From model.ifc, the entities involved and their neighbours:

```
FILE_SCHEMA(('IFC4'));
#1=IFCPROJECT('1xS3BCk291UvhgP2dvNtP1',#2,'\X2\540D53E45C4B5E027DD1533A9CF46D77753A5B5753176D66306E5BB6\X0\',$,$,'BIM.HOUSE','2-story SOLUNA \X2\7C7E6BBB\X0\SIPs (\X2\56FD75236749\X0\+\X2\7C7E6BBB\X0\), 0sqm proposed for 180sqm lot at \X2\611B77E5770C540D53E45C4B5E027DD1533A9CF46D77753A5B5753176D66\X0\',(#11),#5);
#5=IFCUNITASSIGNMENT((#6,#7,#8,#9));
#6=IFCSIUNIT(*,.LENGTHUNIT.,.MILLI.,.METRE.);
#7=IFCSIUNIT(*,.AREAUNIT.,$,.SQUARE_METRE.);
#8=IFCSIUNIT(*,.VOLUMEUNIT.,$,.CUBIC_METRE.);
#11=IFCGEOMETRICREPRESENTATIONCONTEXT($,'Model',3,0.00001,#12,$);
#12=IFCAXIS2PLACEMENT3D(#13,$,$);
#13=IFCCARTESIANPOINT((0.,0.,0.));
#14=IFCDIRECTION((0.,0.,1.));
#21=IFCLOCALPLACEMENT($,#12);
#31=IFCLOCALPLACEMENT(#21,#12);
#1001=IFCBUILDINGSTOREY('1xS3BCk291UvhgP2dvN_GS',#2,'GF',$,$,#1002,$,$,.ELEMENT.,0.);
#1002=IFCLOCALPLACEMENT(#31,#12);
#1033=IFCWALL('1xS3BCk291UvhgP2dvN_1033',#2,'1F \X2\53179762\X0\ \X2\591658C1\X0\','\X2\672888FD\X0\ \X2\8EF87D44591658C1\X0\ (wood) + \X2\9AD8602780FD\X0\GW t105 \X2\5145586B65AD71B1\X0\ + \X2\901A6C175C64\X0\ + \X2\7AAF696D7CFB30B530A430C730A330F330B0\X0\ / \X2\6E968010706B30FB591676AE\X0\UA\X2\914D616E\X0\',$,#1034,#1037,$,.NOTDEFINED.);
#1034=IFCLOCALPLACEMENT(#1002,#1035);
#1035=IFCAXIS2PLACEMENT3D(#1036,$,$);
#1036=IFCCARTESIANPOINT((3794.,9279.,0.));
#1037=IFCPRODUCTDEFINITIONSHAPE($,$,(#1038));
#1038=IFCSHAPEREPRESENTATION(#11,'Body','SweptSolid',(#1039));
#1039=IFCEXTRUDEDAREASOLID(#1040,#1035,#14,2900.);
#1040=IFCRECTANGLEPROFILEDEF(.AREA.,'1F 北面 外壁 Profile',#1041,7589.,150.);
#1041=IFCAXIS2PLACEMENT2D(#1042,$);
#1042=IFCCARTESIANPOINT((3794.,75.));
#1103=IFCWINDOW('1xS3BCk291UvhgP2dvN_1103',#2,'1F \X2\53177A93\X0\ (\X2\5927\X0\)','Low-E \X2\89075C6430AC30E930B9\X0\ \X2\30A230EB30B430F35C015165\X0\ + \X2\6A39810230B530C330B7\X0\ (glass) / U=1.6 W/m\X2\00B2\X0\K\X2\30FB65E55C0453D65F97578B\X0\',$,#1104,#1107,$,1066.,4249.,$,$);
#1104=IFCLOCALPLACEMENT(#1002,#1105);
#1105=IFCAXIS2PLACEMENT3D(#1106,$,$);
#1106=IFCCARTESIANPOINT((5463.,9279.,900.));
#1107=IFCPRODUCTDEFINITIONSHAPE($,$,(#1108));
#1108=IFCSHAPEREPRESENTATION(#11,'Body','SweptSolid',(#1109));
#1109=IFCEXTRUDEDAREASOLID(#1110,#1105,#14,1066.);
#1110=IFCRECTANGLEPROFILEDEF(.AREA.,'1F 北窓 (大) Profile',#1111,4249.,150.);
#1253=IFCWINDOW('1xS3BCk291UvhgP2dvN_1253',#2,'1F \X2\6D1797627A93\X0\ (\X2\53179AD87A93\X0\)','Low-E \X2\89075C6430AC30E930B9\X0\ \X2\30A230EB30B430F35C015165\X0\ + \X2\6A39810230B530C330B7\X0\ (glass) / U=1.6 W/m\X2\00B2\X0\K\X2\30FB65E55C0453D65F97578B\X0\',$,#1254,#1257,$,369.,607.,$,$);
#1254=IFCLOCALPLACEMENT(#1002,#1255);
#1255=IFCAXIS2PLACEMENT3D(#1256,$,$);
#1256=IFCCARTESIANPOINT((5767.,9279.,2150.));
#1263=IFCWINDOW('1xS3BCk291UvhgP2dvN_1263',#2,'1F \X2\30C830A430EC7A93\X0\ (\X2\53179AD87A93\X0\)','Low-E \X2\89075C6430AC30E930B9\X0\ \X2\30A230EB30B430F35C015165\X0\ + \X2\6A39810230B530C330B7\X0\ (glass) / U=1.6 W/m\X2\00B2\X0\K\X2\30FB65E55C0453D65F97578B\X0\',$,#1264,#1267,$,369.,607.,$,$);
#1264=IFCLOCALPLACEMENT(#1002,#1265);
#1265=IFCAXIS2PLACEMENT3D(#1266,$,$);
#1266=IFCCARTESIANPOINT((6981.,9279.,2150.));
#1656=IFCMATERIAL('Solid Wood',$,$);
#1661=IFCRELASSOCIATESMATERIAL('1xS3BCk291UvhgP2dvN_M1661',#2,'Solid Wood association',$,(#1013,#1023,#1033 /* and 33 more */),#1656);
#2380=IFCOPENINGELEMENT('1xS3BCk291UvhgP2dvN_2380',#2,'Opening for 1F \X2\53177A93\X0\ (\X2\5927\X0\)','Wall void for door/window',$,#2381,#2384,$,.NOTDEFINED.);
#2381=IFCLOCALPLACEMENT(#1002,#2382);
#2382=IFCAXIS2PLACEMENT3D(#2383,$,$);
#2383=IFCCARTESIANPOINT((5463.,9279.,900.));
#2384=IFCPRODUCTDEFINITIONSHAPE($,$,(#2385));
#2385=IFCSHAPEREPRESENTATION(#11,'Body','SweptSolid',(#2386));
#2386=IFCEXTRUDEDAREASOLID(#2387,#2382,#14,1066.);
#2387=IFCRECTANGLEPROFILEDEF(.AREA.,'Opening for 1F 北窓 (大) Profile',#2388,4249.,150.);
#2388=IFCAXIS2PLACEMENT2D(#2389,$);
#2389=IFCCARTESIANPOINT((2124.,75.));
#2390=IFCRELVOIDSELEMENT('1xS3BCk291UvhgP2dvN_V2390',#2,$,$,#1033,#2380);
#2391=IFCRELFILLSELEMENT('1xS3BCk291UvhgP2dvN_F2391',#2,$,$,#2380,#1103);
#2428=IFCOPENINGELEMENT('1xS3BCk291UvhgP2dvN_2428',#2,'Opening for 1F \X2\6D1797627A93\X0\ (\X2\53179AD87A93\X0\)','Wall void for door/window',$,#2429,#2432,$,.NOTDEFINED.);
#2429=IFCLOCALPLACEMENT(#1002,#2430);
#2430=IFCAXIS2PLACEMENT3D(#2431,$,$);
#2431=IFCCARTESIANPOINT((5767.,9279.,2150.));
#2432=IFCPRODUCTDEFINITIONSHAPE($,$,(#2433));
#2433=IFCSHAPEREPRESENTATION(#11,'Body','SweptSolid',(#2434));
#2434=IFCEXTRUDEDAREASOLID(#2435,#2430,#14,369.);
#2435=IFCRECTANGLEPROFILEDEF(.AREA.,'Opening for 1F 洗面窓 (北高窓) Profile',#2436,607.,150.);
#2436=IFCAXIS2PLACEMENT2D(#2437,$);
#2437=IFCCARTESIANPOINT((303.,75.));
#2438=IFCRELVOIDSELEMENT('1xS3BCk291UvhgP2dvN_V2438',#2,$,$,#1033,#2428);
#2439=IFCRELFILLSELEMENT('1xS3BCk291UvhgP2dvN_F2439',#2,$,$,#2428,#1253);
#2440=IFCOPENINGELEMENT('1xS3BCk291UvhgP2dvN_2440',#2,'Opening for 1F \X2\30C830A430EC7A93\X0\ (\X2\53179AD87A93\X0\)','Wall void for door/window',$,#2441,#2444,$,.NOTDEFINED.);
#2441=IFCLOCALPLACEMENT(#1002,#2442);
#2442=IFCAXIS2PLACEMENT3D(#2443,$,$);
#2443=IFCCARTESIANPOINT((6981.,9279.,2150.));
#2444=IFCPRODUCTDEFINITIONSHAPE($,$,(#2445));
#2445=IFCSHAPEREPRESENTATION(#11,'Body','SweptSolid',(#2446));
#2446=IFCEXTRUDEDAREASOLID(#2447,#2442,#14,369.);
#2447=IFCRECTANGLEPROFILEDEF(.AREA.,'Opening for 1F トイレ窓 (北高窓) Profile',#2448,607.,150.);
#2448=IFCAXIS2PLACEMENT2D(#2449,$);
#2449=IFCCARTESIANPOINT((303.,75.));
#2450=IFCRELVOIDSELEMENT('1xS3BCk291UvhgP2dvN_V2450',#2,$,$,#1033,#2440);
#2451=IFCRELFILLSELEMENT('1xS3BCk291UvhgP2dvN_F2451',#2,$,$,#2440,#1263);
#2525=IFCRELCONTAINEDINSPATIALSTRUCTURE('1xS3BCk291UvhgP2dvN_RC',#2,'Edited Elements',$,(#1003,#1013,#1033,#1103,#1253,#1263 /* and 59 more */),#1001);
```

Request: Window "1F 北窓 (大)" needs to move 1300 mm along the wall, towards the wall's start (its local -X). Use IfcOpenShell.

```python
import ifcopenshell
import ifcopenshell.api.geometry
import ifcopenshell.util.placement
import ifcopenshell.util.unit

model = ifcopenshell.open("model.ifc")
unit_scale = ifcopenshell.util.unit.calculate_unit_scale(model)

window = model.by_id(1103)
opening = window.FillsVoids[0].RelatingOpeningElement
wall = opening.VoidsElements[0].RelatingBuildingElement

wall_matrix = ifcopenshell.util.placement.get_local_placement(wall.ObjectPlacement)
shift = wall_matrix[:3, 0] * -1.3 / unit_scale
before = ifcopenshell.util.placement.get_local_placement(window.ObjectPlacement)[:3, 3].copy()

# The window is not placed relative to its opening, so move both.
for product in (opening, window):
    matrix = ifcopenshell.util.placement.get_local_placement(product.ObjectPlacement)
    matrix[:3, 3] += shift
    ifcopenshell.api.geometry.edit_object_placement(model, product=product, matrix=matrix, is_si=False)

after = ifcopenshell.util.placement.get_local_placement(window.ObjectPlacement)[:3, 3]
print("window moved by", (after - before).round(3) + 0.0)

model.write("model_edited.ifc")
```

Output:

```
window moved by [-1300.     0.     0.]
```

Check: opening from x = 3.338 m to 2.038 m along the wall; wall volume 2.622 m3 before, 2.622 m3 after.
